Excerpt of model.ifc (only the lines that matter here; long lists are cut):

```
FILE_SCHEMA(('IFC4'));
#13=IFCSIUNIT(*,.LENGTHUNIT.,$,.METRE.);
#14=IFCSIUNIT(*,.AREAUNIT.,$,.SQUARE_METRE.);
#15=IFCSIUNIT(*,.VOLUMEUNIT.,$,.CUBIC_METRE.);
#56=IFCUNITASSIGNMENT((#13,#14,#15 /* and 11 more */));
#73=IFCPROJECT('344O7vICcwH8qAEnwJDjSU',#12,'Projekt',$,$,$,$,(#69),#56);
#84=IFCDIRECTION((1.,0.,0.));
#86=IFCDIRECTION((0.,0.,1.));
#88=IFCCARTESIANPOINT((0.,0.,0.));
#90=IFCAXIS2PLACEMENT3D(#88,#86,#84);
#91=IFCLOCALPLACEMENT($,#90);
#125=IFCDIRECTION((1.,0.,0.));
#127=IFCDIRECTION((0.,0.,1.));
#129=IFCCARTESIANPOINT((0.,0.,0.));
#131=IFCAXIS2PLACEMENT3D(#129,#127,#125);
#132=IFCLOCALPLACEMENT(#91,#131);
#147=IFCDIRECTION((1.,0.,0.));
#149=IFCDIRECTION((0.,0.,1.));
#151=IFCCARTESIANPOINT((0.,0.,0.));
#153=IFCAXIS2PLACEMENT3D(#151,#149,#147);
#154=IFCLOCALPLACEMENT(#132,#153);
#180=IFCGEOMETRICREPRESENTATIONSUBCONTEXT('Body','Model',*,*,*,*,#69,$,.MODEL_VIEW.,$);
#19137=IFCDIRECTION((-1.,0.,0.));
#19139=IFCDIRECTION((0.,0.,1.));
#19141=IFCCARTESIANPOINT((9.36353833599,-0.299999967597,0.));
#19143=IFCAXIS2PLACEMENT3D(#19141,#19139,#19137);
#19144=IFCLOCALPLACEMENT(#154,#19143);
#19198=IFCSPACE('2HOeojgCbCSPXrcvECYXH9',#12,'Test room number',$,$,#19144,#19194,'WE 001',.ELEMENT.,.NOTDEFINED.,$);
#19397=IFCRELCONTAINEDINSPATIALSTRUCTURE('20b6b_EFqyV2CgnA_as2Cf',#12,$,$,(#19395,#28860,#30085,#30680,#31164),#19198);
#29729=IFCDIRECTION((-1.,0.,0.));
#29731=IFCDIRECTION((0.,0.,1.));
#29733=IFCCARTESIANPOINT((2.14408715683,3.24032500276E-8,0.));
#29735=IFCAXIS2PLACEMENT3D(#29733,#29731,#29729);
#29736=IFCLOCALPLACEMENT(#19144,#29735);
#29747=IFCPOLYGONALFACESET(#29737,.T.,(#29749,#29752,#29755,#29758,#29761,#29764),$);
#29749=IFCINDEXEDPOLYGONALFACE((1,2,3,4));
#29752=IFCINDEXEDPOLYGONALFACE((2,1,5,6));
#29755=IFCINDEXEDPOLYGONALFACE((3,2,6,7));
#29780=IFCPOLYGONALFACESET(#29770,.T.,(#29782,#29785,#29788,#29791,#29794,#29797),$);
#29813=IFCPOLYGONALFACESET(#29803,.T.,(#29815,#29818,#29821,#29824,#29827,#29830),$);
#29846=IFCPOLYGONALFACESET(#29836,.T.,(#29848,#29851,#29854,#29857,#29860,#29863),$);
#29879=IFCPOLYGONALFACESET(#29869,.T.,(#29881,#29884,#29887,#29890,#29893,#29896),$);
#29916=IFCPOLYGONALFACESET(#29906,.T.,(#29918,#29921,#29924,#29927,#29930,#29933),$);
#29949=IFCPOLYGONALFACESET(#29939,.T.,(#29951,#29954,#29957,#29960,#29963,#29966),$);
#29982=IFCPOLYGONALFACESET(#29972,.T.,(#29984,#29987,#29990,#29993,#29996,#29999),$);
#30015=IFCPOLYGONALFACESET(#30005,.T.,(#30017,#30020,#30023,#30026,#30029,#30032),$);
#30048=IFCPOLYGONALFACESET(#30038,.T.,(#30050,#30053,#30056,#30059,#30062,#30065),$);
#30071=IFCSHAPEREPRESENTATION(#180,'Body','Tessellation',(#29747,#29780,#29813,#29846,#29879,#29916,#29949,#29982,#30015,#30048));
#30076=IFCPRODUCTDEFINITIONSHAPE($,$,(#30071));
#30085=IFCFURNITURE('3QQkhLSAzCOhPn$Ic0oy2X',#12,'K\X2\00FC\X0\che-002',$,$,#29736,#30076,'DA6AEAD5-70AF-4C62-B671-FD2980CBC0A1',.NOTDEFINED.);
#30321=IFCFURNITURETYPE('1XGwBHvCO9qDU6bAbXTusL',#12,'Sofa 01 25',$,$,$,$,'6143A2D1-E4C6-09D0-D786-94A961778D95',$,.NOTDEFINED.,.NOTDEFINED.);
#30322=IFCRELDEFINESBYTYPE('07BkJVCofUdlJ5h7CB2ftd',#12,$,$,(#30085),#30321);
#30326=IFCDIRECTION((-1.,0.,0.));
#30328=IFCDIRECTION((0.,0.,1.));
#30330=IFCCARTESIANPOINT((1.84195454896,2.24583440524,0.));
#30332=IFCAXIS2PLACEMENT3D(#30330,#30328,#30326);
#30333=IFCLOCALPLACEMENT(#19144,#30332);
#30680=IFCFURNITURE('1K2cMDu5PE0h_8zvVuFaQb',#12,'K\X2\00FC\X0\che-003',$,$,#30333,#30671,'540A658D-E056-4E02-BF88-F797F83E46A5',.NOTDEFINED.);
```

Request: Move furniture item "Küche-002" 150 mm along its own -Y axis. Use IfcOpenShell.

```python
import ifcopenshell
import ifcopenshell.api.geometry
import ifcopenshell.util.placement
import ifcopenshell.util.unit

model = ifcopenshell.open("model.ifc")
unit_scale = ifcopenshell.util.unit.calculate_unit_scale(model)

item = model.by_id(30085)
matrix = ifcopenshell.util.placement.get_local_placement(item.ObjectPlacement)
matrix[:3, 3] -= matrix[:3, 1] * 0.15 / unit_scale
ifcopenshell.api.geometry.edit_object_placement(model, product=item, matrix=matrix, is_si=False)

print(ifcopenshell.util.placement.get_local_placement(item.ObjectPlacement).round(3) + 0.0)

model.write("model_edited.ifc")
```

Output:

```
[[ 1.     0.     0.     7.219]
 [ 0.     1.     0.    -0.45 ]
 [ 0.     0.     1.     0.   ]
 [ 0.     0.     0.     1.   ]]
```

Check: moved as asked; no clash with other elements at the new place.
